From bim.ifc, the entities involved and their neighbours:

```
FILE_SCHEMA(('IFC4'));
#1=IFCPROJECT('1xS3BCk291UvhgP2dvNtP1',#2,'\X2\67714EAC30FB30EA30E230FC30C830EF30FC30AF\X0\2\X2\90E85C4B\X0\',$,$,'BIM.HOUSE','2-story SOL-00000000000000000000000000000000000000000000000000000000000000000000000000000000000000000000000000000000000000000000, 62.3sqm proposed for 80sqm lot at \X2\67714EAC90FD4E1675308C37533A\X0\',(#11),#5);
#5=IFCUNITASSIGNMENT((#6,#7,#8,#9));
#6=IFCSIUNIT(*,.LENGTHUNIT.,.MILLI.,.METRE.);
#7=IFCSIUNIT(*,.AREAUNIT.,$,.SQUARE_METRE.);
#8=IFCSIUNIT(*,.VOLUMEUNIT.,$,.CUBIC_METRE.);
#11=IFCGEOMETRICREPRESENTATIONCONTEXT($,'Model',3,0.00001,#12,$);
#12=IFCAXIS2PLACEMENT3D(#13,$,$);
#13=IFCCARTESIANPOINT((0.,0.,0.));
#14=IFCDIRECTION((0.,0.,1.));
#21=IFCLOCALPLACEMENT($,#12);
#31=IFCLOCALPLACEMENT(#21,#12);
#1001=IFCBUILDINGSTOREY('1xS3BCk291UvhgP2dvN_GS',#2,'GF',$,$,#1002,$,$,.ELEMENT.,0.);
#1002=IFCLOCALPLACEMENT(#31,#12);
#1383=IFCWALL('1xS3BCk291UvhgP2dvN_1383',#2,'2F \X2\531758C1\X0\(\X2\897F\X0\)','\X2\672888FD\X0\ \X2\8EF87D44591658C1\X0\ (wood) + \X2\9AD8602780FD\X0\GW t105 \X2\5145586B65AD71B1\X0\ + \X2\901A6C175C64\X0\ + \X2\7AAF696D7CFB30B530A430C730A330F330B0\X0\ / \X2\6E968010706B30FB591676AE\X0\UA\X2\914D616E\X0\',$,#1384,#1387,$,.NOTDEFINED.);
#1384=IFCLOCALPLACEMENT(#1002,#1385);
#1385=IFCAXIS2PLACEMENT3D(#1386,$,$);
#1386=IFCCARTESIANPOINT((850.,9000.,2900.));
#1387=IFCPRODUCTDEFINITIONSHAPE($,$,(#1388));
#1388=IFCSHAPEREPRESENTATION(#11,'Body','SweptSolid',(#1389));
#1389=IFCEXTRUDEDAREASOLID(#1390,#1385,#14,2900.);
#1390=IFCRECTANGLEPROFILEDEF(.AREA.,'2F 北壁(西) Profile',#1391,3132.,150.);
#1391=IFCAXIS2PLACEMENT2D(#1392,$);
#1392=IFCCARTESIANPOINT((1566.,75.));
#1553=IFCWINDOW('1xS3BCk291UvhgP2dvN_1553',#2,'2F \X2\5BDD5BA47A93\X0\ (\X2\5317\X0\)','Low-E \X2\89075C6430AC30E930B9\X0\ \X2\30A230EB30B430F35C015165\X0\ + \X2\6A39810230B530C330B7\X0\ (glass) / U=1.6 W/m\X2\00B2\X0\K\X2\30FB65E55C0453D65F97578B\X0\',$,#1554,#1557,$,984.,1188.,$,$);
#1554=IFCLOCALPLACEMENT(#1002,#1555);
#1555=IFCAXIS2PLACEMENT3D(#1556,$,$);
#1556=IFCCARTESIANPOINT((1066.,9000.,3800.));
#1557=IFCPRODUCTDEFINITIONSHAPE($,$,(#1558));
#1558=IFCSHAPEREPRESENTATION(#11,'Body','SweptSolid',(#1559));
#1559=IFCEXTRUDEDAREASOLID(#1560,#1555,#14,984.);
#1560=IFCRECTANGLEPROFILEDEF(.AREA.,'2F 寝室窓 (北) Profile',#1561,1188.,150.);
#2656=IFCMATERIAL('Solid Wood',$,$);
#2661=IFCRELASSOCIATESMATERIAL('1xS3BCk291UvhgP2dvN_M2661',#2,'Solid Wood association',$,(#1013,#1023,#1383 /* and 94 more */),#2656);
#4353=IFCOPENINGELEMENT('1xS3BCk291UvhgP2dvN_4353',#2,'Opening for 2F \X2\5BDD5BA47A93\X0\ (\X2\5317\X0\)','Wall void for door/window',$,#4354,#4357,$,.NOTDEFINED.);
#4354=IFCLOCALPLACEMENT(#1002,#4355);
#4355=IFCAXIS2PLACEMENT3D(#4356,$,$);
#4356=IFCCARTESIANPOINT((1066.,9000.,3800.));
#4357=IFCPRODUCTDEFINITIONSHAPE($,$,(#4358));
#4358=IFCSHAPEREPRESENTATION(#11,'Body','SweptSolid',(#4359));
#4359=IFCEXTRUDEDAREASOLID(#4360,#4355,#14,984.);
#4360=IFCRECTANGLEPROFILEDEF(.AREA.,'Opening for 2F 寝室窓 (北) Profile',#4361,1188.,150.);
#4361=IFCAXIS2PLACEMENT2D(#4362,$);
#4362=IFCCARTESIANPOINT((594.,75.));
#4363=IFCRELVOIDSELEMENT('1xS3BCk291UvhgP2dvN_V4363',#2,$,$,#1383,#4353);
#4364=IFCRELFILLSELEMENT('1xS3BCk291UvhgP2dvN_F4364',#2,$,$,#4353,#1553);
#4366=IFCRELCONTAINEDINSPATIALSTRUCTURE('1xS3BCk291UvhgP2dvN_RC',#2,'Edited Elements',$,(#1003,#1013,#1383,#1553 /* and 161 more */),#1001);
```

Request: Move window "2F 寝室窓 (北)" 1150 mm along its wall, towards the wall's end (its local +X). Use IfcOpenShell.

```python
import ifcopenshell
import ifcopenshell.api.geometry
import ifcopenshell.util.placement
import ifcopenshell.util.unit

model = ifcopenshell.open("bim.ifc")
unit_scale = ifcopenshell.util.unit.calculate_unit_scale(model)

window = model.by_guid("1xS3BCk291UvhgP2dvN_1553")
opening = window.FillsVoids[0].RelatingOpeningElement
wall = opening.VoidsElements[0].RelatingBuildingElement

wall_matrix = ifcopenshell.util.placement.get_local_placement(wall.ObjectPlacement)
shift = wall_matrix[:3, 0] * 1.15 / unit_scale
before = ifcopenshell.util.placement.get_local_placement(window.ObjectPlacement)[:3, 3].copy()

# The window is not placed relative to its opening, so move both.
for product in (opening, window):
    matrix = ifcopenshell.util.placement.get_local_placement(product.ObjectPlacement)
    matrix[:3, 3] += shift
    ifcopenshell.api.geometry.edit_object_placement(model, product=product, matrix=matrix, is_si=False)

after = ifcopenshell.util.placement.get_local_placement(window.ObjectPlacement)[:3, 3]
print("window moved by", (after - before).round(3) + 0.0)

model.write("bim_v2.ifc")
```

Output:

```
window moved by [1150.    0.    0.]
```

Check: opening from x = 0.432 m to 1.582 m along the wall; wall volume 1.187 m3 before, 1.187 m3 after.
